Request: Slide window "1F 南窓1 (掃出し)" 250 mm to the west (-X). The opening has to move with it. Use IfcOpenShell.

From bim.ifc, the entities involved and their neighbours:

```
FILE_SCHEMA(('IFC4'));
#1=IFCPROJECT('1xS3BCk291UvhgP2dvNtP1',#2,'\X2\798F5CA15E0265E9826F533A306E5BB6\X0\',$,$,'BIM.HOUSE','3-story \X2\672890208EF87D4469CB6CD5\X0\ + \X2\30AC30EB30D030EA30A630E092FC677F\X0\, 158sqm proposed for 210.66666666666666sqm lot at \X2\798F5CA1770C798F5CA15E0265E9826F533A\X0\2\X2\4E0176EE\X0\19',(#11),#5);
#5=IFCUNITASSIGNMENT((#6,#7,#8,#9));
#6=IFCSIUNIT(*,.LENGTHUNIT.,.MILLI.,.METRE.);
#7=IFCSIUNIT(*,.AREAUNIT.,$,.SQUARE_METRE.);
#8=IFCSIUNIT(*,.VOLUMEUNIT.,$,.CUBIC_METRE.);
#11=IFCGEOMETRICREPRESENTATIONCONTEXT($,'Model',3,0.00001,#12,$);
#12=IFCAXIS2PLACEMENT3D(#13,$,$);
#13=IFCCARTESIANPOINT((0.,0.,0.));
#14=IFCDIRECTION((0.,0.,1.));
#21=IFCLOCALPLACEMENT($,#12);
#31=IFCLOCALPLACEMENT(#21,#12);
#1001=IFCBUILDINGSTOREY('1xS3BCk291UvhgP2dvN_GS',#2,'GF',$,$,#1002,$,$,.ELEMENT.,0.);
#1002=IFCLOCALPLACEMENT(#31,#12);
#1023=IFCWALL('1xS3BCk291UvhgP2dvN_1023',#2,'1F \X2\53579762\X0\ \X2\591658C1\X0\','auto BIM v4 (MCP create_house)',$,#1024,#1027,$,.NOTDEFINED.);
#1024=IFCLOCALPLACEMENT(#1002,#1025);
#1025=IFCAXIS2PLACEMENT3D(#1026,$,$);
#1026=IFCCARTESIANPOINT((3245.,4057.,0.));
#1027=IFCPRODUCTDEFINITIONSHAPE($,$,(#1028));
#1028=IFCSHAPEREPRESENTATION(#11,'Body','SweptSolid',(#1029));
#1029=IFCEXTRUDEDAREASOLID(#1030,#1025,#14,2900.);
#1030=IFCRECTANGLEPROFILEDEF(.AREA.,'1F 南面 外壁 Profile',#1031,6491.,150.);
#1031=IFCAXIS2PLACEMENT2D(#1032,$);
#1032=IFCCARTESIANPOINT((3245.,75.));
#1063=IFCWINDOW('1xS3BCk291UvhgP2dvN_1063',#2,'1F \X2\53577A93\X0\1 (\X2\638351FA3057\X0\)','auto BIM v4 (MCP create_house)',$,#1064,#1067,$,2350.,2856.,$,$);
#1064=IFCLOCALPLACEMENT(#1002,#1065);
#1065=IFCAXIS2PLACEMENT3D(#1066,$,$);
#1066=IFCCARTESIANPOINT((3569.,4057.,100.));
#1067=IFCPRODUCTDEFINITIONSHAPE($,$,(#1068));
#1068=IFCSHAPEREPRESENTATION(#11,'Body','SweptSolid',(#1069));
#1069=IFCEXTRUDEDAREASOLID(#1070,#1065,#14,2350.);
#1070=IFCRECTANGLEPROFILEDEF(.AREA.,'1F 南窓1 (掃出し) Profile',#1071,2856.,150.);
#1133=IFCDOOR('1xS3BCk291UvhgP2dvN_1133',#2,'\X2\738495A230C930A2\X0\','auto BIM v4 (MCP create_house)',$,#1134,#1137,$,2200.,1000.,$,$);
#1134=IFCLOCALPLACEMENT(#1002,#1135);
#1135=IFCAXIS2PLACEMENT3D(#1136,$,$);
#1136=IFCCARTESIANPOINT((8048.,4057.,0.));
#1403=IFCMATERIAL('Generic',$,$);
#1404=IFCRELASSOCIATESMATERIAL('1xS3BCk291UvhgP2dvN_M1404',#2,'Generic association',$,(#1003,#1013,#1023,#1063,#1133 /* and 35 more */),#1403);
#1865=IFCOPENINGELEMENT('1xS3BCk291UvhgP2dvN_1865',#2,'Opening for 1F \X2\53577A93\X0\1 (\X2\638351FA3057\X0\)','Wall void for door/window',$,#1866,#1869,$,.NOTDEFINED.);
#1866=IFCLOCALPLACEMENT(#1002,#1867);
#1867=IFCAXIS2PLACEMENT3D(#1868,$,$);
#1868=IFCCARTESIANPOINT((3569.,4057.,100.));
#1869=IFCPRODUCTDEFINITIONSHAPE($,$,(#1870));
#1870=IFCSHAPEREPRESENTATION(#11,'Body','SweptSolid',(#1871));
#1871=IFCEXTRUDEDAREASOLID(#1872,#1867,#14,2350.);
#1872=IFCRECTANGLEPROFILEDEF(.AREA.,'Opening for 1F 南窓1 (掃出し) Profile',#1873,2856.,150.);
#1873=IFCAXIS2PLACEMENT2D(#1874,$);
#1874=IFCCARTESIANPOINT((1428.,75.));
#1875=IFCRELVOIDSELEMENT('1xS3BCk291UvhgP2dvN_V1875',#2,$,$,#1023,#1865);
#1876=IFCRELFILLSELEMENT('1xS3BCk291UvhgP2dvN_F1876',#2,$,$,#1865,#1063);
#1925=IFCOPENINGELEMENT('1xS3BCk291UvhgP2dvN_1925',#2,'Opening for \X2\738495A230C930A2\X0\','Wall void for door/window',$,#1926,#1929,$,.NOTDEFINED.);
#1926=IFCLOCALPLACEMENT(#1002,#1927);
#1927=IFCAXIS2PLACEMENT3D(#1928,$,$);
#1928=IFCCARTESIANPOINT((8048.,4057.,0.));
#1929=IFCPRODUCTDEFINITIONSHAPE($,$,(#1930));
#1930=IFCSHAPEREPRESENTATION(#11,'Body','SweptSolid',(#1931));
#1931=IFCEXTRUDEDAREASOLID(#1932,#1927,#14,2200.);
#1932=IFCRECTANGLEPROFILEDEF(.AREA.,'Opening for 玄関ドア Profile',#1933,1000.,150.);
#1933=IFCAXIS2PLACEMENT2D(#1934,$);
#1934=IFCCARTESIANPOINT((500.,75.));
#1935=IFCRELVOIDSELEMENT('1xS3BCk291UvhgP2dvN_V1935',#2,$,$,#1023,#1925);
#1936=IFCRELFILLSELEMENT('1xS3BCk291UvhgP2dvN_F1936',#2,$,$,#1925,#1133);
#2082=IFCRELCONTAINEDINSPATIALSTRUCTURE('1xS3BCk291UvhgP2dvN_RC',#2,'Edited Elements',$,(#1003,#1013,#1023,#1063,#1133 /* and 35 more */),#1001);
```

```python
import ifcopenshell
import ifcopenshell.api.geometry
import ifcopenshell.util.placement
import ifcopenshell.util.unit

model = ifcopenshell.open("bim.ifc")
unit_scale = ifcopenshell.util.unit.calculate_unit_scale(model)

window = model.by_guid("1xS3BCk291UvhgP2dvN_1063")
opening = window.FillsVoids[0].RelatingOpeningElement
wall = opening.VoidsElements[0].RelatingBuildingElement

wall_matrix = ifcopenshell.util.placement.get_local_placement(wall.ObjectPlacement)
shift = wall_matrix[:3, 0] * -0.25 / unit_scale
before = ifcopenshell.util.placement.get_local_placement(window.ObjectPlacement)[:3, 3].copy()

# The window is not placed relative to its opening, so move both.
for product in (opening, window):
    matrix = ifcopenshell.util.placement.get_local_placement(product.ObjectPlacement)
    matrix[:3, 3] += shift
    ifcopenshell.api.geometry.edit_object_placement(model, product=product, matrix=matrix, is_si=False)

after = ifcopenshell.util.placement.get_local_placement(window.ObjectPlacement)[:3, 3]
print("window moved by", (after - before).round(3) + 0.0)

model.write("bim_rev.ifc")
```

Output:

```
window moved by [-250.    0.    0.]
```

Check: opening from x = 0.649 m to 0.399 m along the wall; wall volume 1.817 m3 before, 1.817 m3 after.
